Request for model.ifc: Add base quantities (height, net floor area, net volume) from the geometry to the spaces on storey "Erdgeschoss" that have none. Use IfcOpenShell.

First a look at what the model holds.

```python
import ifcopenshell
import ifcopenshell.util.element
import ifcopenshell.util.unit

model = ifcopenshell.open("model.ifc")
print(model.schema)
for unit_type in ("LENGTHUNIT", "AREAUNIT", "VOLUMEUNIT"):
    print(unit_type, ifcopenshell.util.unit.calculate_unit_scale(model, unit_type))
storey = next(s for s in model.by_type("IfcBuildingStorey") if s.Name == "Erdgeschoss")
spaces = [e for e in ifcopenshell.util.element.get_decomposition(storey) if e.is_a("IfcSpace")]
for e in sorted(spaces, key=lambda e: e.id()):
    print(e.id(), e.is_a(), e.Name, list(ifcopenshell.util.element.get_psets(e, qtos_only=True)), sep=" | ")
```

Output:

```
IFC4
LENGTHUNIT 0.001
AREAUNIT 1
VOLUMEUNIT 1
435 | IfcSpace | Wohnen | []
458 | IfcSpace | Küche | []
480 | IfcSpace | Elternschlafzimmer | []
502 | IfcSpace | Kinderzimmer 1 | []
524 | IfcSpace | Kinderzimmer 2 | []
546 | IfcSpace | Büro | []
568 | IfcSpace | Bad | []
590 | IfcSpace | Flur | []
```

```python
import ifcopenshell
import ifcopenshell.api.pset
import ifcopenshell.geom
import ifcopenshell.util.element
import ifcopenshell.util.shape
import ifcopenshell.util.unit

model = ifcopenshell.open("model.ifc")
unit_scale = ifcopenshell.util.unit.calculate_unit_scale(model)
area_scale = ifcopenshell.util.unit.calculate_unit_scale(model, "AREAUNIT")
volume_scale = ifcopenshell.util.unit.calculate_unit_scale(model, "VOLUMEUNIT")
settings = ifcopenshell.geom.settings()

storey = next(s for s in model.by_type("IfcBuildingStorey") if s.Name == "Erdgeschoss")
spaces = [e for e in ifcopenshell.util.element.get_decomposition(storey) if e.is_a("IfcSpace")]

for e in sorted(spaces, key=lambda e: e.id()):
    if ifcopenshell.util.element.get_psets(e, qtos_only=True, should_inherit=False):
        continue
    # Geometry comes back in metres, in the element's own axes.
    shape = ifcopenshell.geom.create_shape(settings, e)
    values = {
        "Height": ifcopenshell.util.shape.get_z(shape.geometry) / unit_scale,
        "NetFloorArea": ifcopenshell.util.shape.get_footprint_area(shape.geometry) / area_scale,
        "NetVolume": ifcopenshell.util.shape.get_volume(shape.geometry) / volume_scale,
    }
    qto = ifcopenshell.api.pset.add_qto(model, product=e, name="Qto_SpaceBaseQuantities")
    ifcopenshell.api.pset.edit_qto(model, qto=qto, properties=values)
    print(e.id(), {k: round(v, 3) for k, v in values.items()})

model.write("model_rev.ifc")
```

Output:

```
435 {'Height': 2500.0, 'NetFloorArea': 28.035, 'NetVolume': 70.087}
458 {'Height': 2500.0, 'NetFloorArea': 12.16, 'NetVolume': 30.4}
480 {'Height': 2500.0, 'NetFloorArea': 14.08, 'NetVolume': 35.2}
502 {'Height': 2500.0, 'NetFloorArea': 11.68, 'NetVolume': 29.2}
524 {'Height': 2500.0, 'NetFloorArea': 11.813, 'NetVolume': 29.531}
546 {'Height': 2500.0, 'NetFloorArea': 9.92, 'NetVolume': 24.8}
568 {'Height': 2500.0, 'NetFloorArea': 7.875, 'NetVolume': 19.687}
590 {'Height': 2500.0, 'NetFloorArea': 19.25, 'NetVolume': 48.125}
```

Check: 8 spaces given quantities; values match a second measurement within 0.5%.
